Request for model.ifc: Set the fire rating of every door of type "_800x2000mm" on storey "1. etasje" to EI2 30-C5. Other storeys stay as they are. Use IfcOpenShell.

First a look at what the model holds.

```python
import ifcopenshell
import ifcopenshell.util.element

model = ifcopenshell.open("model.ifc")
print(model.schema)
storey = next(s for s in model.by_type("IfcBuildingStorey") if s.Name == "1. etasje")
doors = [e for e in ifcopenshell.util.element.get_decomposition(storey) if e.is_a("IfcDoor")]
seen = {}
for e in doors:
    element_type = ifcopenshell.util.element.get_type(e)
    key = (element_type.Name if element_type != e and element_type else None, ifcopenshell.util.element.get_pset(e, "Pset_DoorCommon", "FireRating"))
    seen[key] = seen.get(key, 0) + 1
for (name, value), count in sorted(seen.items(), key=str):
    print(count, "x", name, "|", value)
```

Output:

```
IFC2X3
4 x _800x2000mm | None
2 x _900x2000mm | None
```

```python
import ifcopenshell
import ifcopenshell.api.pset
import ifcopenshell.util.element

model = ifcopenshell.open("model.ifc")

storey = next(s for s in model.by_type("IfcBuildingStorey") if s.Name == "1. etasje")
doors = [e for e in ifcopenshell.util.element.get_decomposition(storey) if e.is_a("IfcDoor")]

count = 0
for e in doors:
    element_type = ifcopenshell.util.element.get_type(e)
    if element_type in (None, e) or element_type.Name != "_800x2000mm":
        continue
    # add_pset returns the element's existing set when there is one.
    pset = ifcopenshell.api.pset.add_pset(model, product=e, name="Pset_DoorCommon")
    ifcopenshell.api.pset.edit_pset(model, pset=pset, properties={"FireRating": "EI2 30-C5"})
    count += 1

print(count, "doors updated")

model.write("model-out.ifc")
```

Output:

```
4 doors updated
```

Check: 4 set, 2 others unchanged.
